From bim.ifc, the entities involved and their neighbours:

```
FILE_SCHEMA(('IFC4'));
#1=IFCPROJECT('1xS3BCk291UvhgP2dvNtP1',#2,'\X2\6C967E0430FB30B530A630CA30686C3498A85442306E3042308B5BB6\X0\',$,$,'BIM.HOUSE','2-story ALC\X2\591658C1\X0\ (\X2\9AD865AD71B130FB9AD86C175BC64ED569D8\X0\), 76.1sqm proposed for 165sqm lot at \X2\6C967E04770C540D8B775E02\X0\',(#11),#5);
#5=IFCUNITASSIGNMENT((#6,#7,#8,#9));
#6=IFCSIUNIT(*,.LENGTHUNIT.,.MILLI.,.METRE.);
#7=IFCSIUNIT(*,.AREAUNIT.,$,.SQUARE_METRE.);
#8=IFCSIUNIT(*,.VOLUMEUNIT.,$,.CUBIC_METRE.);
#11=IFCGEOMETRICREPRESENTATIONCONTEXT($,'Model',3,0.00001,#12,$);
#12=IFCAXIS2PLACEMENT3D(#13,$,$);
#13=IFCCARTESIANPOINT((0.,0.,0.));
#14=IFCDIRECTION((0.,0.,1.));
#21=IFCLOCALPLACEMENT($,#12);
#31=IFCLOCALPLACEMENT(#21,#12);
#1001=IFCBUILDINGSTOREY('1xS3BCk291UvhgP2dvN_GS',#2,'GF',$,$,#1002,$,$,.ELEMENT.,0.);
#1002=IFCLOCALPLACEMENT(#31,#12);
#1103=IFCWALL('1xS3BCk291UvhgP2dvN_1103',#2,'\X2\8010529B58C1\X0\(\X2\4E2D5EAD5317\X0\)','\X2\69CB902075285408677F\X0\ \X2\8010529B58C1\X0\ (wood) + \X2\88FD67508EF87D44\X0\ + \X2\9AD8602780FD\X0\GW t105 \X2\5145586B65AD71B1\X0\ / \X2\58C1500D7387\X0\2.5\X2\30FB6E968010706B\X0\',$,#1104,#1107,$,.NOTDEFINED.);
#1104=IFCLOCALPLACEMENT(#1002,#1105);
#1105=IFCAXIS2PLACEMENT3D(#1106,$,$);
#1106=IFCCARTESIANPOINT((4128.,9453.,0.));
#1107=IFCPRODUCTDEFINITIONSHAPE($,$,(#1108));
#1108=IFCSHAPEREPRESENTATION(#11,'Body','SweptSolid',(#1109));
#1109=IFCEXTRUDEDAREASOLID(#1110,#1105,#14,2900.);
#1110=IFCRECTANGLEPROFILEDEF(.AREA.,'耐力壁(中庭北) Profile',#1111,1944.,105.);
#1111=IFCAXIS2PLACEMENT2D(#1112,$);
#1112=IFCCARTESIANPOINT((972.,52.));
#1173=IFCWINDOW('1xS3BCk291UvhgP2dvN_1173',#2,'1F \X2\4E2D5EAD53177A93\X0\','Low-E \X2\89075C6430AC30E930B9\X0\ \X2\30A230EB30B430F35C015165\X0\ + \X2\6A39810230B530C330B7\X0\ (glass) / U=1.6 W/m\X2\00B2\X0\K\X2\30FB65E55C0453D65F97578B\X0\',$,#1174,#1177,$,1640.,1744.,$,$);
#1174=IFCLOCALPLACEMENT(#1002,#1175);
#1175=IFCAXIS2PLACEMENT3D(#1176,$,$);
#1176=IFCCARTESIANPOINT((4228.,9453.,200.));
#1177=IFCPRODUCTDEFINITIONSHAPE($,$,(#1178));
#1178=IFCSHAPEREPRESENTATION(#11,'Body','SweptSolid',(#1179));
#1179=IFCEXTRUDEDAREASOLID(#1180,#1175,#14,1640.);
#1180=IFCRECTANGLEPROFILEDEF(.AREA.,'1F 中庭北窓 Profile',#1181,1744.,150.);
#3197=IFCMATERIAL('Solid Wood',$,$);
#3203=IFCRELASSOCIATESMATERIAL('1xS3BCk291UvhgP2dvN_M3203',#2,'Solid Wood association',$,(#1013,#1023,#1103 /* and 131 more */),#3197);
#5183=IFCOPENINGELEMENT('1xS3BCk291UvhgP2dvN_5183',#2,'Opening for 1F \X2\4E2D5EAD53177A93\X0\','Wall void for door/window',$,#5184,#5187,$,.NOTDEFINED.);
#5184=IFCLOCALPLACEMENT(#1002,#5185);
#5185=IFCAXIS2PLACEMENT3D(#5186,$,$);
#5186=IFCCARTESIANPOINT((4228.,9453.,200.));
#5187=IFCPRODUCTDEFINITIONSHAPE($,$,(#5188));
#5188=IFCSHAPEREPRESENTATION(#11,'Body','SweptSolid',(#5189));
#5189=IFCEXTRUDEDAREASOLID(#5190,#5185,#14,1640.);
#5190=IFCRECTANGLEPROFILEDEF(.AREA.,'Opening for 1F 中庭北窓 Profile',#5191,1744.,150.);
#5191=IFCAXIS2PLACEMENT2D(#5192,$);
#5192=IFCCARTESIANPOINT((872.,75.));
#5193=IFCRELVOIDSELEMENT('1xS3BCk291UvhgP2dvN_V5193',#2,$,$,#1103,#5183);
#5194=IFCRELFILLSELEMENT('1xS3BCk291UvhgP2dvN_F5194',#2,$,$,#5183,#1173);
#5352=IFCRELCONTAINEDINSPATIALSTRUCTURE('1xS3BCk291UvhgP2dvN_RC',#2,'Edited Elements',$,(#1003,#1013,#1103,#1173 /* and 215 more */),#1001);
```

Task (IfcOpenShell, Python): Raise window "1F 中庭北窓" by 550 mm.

```python
import numpy as np
import ifcopenshell
import ifcopenshell.api.geometry
import ifcopenshell.util.placement
import ifcopenshell.util.unit

model = ifcopenshell.open("bim.ifc")
unit_scale = ifcopenshell.util.unit.calculate_unit_scale(model)

window = model.by_guid("1xS3BCk291UvhgP2dvN_1173")
opening = window.FillsVoids[0].RelatingOpeningElement
dz = 0.55 / unit_scale

shift = np.array([0.0, 0.0, dz])
# The window is not placed relative to its opening, so move both.
for product in (opening, window):
    matrix = ifcopenshell.util.placement.get_local_placement(product.ObjectPlacement)
    matrix[:3, 3] += shift
    ifcopenshell.api.geometry.edit_object_placement(model, product=product, matrix=matrix, is_si=False)

print(f"moved by {dz * unit_scale:+.3f} m")

model.write("bim_rev.ifc")
```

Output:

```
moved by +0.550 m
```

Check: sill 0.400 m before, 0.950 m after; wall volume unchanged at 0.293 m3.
